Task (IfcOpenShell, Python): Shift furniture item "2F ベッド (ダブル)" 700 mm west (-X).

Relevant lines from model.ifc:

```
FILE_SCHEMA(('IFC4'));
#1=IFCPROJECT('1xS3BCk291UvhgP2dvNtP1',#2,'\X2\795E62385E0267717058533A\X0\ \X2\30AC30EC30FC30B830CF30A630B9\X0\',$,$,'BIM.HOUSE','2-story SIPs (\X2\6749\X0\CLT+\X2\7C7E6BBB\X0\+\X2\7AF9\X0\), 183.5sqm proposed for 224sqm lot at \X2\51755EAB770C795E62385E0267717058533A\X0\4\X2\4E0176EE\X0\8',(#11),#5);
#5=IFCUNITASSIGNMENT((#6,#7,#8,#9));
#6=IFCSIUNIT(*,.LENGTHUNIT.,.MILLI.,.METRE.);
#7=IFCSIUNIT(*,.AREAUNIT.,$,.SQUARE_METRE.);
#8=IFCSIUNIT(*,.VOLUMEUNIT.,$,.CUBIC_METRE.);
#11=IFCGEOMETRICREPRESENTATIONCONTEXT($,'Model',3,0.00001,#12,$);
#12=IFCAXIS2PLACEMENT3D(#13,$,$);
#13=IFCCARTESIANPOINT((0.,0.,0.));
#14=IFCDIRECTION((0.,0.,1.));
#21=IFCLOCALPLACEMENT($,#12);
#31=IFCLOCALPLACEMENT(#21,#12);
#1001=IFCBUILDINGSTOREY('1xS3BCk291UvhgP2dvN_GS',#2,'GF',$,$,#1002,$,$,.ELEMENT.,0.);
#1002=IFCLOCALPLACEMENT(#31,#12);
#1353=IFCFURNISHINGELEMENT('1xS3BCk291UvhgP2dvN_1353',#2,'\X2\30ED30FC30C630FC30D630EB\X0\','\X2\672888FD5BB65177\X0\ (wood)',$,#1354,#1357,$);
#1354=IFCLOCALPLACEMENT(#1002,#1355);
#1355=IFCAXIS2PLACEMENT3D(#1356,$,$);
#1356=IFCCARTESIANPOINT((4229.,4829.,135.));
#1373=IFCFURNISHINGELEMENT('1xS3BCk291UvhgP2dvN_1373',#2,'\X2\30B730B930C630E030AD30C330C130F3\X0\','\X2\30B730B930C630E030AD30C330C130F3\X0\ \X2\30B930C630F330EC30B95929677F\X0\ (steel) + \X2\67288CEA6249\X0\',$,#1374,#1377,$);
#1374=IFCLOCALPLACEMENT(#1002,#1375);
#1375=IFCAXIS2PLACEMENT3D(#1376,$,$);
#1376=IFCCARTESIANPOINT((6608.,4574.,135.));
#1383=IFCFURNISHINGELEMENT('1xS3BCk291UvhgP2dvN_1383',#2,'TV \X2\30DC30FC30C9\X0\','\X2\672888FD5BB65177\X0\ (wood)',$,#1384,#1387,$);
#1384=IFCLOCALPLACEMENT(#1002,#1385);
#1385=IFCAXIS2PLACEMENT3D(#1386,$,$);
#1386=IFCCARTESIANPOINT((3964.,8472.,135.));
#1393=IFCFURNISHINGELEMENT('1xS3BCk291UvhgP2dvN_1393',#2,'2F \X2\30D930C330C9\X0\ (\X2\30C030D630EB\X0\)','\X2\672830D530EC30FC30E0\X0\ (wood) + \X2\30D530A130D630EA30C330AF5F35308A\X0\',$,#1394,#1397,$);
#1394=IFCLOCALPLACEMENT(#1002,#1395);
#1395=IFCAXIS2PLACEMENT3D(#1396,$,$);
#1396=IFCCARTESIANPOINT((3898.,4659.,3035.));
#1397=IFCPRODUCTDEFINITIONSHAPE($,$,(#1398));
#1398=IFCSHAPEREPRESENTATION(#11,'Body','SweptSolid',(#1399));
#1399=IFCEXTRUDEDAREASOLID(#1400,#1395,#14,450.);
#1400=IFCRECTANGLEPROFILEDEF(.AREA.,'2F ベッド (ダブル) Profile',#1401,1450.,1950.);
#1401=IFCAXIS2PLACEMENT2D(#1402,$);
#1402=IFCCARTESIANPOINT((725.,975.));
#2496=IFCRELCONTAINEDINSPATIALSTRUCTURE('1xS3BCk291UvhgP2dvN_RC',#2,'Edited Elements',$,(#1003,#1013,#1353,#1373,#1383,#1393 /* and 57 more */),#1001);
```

```python
import ifcopenshell
import ifcopenshell.api.geometry
import ifcopenshell.util.placement

model = ifcopenshell.open("model.ifc")

item = model.by_id(1393)
matrix = ifcopenshell.util.placement.get_local_placement(item.ObjectPlacement)
matrix[0, 3] -= 700.0
ifcopenshell.api.geometry.edit_object_placement(model, product=item, matrix=matrix, is_si=False)

print(ifcopenshell.util.placement.get_local_placement(item.ObjectPlacement).round(3) + 0.0)

model.write("model_rev.ifc")
```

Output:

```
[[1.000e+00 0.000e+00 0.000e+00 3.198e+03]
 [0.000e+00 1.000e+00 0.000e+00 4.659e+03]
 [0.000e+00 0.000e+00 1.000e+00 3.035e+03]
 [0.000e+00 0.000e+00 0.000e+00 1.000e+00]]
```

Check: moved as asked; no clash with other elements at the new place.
